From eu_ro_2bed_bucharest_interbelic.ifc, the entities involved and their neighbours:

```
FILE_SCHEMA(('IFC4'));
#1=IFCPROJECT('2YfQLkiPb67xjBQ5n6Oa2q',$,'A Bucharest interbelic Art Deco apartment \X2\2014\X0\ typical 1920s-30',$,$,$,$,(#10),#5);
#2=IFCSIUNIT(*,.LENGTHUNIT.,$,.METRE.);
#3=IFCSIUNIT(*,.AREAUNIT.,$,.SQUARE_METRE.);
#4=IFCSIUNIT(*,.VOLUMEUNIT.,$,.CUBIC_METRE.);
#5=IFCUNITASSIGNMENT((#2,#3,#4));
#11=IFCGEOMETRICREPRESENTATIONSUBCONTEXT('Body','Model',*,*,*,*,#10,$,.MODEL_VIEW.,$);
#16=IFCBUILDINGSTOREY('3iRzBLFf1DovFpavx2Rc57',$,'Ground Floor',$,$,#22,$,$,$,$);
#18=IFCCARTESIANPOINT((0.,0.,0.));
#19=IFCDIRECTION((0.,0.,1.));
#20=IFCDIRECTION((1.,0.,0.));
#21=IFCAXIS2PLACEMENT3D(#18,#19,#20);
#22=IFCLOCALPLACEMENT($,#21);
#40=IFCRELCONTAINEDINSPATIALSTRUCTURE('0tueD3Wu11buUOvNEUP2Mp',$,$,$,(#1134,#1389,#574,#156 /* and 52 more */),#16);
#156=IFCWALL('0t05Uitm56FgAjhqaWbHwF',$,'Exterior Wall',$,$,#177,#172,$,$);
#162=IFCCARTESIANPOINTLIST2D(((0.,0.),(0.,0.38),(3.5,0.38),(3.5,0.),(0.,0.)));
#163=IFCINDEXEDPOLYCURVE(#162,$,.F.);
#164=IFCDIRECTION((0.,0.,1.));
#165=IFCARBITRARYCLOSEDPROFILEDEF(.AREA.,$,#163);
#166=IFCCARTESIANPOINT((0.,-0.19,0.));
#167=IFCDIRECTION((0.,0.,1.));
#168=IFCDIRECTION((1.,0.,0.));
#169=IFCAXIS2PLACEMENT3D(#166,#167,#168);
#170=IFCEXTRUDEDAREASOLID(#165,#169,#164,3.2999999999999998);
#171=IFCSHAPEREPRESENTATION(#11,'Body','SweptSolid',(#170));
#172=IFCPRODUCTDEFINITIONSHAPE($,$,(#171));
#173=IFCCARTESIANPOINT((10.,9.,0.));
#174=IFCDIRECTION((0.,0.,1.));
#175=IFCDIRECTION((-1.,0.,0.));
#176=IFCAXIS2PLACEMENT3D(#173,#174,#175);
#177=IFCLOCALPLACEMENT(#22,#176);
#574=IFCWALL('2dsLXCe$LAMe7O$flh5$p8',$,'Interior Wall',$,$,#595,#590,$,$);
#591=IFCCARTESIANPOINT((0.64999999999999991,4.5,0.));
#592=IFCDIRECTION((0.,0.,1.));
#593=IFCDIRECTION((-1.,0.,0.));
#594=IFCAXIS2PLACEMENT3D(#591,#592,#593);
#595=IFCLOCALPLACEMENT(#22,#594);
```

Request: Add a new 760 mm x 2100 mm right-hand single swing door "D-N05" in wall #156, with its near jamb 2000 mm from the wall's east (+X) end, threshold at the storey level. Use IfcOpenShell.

```python
import numpy as np
import ifcopenshell
import ifcopenshell.api.feature
import ifcopenshell.api.geometry
import ifcopenshell.api.root
import ifcopenshell.api.spatial
import ifcopenshell.geom
import ifcopenshell.util.element
import ifcopenshell.util.placement
import ifcopenshell.util.representation
import ifcopenshell.util.shape
import ifcopenshell.util.unit

model = ifcopenshell.open("eu_ro_2bed_bucharest_interbelic.ifc")
unit_scale = ifcopenshell.util.unit.calculate_unit_scale(model)
settings = ifcopenshell.geom.settings()


def volume(element):
    """Net volume in cubic metres, openings subtracted."""
    shape = ifcopenshell.geom.create_shape(settings, element)
    return ifcopenshell.util.shape.get_volume(shape.geometry)


wall = model.by_id(156)
storey = ifcopenshell.util.element.get_container(wall, ifc_class="IfcBuildingStorey")
context = ifcopenshell.util.representation.get_context(model, "Model", "Body", "MODEL_VIEW")
before = volume(wall)

width, height, from_end, sill = 0.76, 2.1, 2, 0.0  # metres

# The wall runs along its own X axis, and the end named is its -X end.
wall_shape = ifcopenshell.geom.create_shape(settings, wall)
x, y, z = ifcopenshell.util.shape.get_vertices(wall_shape.geometry).T
start = x.min() + from_end
face, thickness = float(y.min()), float(y.max() - y.min())
wall_matrix = ifcopenshell.util.placement.get_local_placement(wall.ObjectPlacement)
level = ifcopenshell.util.placement.get_local_placement(storey.ObjectPlacement)[2, 3]


def in_wall(x, y):
    """Placement at x, y metres in the wall's axes, at sill height."""
    matrix = wall_matrix.copy()
    matrix[:, 3] = wall_matrix @ np.array([x / unit_scale, y / unit_scale, 0.0, 1.0])
    matrix[2, 3] = level + sill / unit_scale
    return matrix


# Opening: a box that overshoots both wall faces by 50 mm.
opening = ifcopenshell.api.root.create_entity(model, ifc_class="IfcOpeningElement", predefined_type="OPENING")
box = ifcopenshell.api.geometry.add_wall_representation(
    model, context=context, length=width, height=height, thickness=thickness + 0.1
)
ifcopenshell.api.geometry.assign_representation(model, product=opening, representation=box)
ifcopenshell.api.geometry.edit_object_placement(model, product=opening, matrix=in_wall(start, face - 0.05), is_si=False)
ifcopenshell.api.feature.add_feature(model, feature=opening, element=wall)

door = ifcopenshell.api.root.create_entity(model, ifc_class="IfcDoor", name="D-N05", predefined_type="DOOR")
door.OverallWidth, door.OverallHeight = width / unit_scale, height / unit_scale
door.OperationType = "SINGLE_SWING_RIGHT"
body = ifcopenshell.api.geometry.add_door_representation(
    model,
    context=context,
    overall_width=door.OverallWidth,
    overall_height=door.OverallHeight,
    operation_type="SINGLE_SWING_RIGHT",
    lining_properties={"LiningDepth": thickness / unit_scale, "ThresholdDepth": thickness / unit_scale},
)
ifcopenshell.api.geometry.assign_representation(model, product=door, representation=body)
ifcopenshell.api.spatial.assign_container(model, products=[door], relating_structure=storey)
ifcopenshell.api.feature.add_filling(model, opening=opening, element=door)

# The lining spans the wall, so the door starts at the wall face.
ifcopenshell.api.geometry.edit_object_placement(model, product=door, matrix=in_wall(start, face), is_si=False)

after = volume(wall)

print(f"wall volume {before:.3f} -> {after:.3f} m3")

model.write("eu_ro_2bed_bucharest_interbelic_v2.ifc")
```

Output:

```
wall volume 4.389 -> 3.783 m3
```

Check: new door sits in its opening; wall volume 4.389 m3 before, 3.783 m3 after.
